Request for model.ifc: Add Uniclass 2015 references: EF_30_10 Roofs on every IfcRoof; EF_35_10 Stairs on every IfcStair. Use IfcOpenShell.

First a look at what the model holds.

```python
import ifcopenshell

model = ifcopenshell.open("model.ifc")
print(model.schema)
print("classifications:", [c.Name for c in model.by_type("IfcClassification")])
for ifc_class in ("IfcDoor", "IfcRoof", "IfcStair", "IfcWall", "IfcWindow"):
    print(ifc_class, len(model.by_type(ifc_class)))
```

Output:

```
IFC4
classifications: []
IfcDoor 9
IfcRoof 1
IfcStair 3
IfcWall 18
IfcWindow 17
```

```python
import ifcopenshell
import ifcopenshell.api.classification

model = ifcopenshell.open("model.ifc")

system = ifcopenshell.api.classification.add_classification(model, classification="Uniclass 2015")

codes = {
    "IfcRoof": ("EF_30_10", "Roofs"),
    "IfcStair": ("EF_35_10", "Stairs"),
}
for ifc_class, (code, name) in codes.items():
    products = model.by_type(ifc_class)
    ifcopenshell.api.classification.add_reference(
        model, products=products, classification=system, identification=code, name=name
    )
    print(code, len(products))

model.write("model-out.ifc")
```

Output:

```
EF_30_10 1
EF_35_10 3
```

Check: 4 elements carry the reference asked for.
